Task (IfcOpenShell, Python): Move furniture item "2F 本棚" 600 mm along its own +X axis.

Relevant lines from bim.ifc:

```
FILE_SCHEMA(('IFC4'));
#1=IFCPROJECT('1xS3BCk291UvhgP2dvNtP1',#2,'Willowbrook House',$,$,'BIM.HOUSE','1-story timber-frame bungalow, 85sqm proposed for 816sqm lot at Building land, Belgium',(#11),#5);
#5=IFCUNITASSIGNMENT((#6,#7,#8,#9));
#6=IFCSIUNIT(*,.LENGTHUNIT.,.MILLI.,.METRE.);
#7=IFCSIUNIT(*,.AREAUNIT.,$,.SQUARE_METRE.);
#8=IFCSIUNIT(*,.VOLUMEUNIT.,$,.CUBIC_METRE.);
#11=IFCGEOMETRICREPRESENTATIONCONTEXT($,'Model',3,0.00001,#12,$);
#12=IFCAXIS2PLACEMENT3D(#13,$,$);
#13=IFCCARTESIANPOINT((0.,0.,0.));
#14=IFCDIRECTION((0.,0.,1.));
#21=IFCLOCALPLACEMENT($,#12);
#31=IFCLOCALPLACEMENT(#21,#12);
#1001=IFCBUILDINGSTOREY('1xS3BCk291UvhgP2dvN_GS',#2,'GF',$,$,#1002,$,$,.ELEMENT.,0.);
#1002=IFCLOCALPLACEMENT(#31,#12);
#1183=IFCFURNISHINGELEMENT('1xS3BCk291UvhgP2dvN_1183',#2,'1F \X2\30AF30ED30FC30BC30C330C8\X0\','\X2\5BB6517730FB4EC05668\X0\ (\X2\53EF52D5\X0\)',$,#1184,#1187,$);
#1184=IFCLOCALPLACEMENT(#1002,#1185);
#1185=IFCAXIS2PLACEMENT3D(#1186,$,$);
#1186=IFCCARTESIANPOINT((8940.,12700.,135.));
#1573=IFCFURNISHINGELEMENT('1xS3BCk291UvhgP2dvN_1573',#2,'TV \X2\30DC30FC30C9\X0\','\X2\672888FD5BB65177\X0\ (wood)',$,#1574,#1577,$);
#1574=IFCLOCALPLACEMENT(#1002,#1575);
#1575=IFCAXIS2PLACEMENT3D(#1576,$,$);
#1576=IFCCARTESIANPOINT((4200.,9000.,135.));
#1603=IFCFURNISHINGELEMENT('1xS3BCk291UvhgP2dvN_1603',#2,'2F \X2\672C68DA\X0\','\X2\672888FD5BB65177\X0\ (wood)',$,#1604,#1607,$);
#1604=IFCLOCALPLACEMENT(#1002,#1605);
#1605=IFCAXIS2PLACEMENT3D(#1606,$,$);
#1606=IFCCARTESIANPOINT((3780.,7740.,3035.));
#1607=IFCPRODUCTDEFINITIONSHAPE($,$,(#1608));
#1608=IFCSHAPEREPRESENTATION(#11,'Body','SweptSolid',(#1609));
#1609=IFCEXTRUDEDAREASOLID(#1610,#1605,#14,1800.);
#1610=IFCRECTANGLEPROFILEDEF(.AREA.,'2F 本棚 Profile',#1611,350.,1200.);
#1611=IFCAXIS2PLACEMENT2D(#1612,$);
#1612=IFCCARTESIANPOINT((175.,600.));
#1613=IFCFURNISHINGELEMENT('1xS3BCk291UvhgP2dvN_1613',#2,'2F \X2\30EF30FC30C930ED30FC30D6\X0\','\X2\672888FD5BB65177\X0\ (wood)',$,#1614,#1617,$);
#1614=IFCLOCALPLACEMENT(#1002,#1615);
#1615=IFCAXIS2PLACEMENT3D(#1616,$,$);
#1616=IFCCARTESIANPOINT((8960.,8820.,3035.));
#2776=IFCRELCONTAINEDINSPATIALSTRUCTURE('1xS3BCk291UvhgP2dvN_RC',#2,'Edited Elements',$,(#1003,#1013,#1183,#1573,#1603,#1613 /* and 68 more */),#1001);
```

```python
import ifcopenshell
import ifcopenshell.api.geometry
import ifcopenshell.util.placement

model = ifcopenshell.open("bim.ifc")

item = model.by_id(1603)
matrix = ifcopenshell.util.placement.get_local_placement(item.ObjectPlacement)
matrix[:3, 3] += matrix[:3, 0] * 600.0
ifcopenshell.api.geometry.edit_object_placement(model, product=item, matrix=matrix, is_si=False)

print(ifcopenshell.util.placement.get_local_placement(item.ObjectPlacement).round(3) + 0.0)

model.write("bim_rev.ifc")
```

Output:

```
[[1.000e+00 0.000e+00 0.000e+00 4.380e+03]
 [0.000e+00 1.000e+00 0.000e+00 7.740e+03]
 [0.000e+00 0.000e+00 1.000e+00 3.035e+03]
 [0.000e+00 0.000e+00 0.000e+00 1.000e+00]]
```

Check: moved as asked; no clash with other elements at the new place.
